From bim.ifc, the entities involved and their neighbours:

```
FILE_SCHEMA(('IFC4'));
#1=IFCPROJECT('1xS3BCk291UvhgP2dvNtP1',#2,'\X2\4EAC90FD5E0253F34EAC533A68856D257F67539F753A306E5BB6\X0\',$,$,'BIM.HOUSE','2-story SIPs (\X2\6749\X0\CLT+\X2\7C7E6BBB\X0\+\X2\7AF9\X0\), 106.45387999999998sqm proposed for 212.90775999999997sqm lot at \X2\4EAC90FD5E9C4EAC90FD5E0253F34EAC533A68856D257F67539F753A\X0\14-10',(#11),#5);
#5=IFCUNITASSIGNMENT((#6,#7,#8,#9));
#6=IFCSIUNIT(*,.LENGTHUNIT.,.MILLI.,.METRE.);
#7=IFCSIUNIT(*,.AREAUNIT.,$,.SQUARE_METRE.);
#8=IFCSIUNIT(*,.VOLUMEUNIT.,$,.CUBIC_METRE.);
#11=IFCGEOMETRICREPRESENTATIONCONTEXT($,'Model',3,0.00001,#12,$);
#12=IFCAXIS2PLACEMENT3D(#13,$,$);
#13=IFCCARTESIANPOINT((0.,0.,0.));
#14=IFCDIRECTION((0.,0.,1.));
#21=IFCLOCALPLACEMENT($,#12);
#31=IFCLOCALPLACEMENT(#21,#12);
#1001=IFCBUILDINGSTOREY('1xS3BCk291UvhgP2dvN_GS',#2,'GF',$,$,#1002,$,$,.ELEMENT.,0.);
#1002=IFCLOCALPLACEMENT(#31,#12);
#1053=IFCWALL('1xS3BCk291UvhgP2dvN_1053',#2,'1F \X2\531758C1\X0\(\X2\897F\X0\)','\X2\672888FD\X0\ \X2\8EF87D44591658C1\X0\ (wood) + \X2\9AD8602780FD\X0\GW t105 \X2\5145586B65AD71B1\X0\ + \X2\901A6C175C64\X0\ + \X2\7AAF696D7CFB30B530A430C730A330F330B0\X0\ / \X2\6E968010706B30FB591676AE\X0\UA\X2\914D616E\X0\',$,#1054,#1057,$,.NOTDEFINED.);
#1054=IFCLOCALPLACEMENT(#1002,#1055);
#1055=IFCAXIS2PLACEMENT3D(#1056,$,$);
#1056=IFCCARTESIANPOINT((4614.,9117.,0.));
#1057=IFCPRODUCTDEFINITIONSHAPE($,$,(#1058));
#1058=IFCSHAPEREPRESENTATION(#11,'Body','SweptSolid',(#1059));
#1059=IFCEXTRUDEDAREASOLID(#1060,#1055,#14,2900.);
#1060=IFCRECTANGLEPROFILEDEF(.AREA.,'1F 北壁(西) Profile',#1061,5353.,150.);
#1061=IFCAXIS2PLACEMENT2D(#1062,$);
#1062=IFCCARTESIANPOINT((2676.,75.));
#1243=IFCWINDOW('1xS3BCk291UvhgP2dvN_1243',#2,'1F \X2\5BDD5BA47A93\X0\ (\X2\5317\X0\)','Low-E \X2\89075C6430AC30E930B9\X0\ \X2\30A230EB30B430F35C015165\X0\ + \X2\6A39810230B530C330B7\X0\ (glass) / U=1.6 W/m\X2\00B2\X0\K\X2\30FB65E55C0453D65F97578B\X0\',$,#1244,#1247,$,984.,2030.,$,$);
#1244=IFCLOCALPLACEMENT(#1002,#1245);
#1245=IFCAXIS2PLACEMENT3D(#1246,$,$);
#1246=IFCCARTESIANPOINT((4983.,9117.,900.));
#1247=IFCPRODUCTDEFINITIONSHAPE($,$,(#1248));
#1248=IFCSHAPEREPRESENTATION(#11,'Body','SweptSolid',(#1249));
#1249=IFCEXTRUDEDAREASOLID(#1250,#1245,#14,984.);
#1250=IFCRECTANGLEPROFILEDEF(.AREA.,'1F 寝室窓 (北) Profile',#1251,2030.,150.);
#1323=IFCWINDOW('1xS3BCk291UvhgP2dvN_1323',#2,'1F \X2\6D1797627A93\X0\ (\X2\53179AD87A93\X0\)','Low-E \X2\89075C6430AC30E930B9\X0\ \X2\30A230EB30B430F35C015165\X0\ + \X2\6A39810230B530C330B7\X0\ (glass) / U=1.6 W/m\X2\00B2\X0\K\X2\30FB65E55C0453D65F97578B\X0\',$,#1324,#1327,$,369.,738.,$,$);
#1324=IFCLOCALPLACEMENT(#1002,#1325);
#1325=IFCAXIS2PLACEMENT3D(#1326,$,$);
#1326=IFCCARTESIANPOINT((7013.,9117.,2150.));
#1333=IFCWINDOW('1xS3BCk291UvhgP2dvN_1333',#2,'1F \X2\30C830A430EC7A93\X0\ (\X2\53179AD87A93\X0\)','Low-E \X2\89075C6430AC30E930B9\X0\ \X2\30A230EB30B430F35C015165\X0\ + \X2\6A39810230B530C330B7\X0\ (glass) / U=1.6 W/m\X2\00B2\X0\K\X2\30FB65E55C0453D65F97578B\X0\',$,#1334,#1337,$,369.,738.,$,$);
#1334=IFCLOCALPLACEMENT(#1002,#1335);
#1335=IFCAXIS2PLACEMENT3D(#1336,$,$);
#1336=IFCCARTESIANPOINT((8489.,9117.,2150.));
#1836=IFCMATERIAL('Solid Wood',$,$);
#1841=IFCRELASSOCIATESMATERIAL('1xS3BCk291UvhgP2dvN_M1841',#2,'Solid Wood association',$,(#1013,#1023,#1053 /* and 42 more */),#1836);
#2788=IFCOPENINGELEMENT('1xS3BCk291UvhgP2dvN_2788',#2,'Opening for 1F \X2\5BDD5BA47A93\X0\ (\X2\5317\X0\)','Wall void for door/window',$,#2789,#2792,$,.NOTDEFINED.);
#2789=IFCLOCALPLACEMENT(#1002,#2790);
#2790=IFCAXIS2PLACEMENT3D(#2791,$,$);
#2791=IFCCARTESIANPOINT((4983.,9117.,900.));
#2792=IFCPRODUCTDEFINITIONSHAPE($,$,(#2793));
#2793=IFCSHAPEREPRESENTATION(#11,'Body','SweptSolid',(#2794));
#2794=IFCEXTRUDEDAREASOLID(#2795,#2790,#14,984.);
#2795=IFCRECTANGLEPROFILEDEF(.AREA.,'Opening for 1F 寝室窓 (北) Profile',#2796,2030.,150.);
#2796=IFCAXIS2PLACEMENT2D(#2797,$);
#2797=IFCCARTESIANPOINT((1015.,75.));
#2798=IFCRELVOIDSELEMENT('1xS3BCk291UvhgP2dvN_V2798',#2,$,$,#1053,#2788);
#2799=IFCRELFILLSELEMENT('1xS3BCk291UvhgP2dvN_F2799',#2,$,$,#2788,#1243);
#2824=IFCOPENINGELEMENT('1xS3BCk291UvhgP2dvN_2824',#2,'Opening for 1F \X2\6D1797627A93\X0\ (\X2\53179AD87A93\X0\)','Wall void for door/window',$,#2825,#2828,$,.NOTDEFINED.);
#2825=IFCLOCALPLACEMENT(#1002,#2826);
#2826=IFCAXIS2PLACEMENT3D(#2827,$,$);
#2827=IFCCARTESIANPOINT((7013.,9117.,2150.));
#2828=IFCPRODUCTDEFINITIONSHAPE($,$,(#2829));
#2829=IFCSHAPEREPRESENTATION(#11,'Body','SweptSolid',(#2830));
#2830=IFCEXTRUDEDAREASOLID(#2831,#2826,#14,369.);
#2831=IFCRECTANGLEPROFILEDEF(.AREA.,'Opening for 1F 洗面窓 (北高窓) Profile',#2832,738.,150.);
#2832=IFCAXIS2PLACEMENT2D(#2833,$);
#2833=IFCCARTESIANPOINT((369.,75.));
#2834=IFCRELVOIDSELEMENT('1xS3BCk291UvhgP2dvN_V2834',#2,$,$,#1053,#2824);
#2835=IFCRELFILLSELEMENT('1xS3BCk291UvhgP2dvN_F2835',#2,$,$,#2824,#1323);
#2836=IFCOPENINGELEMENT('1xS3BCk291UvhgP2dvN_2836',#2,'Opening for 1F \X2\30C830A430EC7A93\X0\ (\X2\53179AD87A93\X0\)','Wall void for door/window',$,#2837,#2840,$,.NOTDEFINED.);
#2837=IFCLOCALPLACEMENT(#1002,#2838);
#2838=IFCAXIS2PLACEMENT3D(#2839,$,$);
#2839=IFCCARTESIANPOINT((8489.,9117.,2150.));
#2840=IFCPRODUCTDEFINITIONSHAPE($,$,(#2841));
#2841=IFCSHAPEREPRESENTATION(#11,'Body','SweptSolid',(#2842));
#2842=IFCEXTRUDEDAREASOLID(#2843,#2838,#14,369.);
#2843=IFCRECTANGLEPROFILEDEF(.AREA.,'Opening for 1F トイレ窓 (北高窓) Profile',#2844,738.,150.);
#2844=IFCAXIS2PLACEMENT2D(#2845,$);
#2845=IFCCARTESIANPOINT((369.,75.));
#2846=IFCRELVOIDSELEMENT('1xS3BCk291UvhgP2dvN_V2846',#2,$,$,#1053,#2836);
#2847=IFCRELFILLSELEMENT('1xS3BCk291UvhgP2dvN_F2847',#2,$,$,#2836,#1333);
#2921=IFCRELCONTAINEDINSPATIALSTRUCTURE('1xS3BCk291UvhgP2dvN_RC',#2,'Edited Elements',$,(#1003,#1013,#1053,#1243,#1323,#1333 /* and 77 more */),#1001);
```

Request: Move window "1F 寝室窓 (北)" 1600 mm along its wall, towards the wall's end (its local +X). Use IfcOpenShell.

```python
import ifcopenshell
import ifcopenshell.api.geometry
import ifcopenshell.util.placement
import ifcopenshell.util.unit

model = ifcopenshell.open("bim.ifc")
unit_scale = ifcopenshell.util.unit.calculate_unit_scale(model)

window = model.by_guid("1xS3BCk291UvhgP2dvN_1243")
opening = window.FillsVoids[0].RelatingOpeningElement
wall = opening.VoidsElements[0].RelatingBuildingElement

wall_matrix = ifcopenshell.util.placement.get_local_placement(wall.ObjectPlacement)
shift = wall_matrix[:3, 0] * 1.6 / unit_scale
before = ifcopenshell.util.placement.get_local_placement(window.ObjectPlacement)[:3, 3].copy()

# The window is not placed relative to its opening, so move both.
for product in (opening, window):
    matrix = ifcopenshell.util.placement.get_local_placement(product.ObjectPlacement)
    matrix[:3, 3] += shift
    ifcopenshell.api.geometry.edit_object_placement(model, product=product, matrix=matrix, is_si=False)

after = ifcopenshell.util.placement.get_local_placement(window.ObjectPlacement)[:3, 3]
print("window moved by", (after - before).round(3) + 0.0)

model.write("bim_updated.ifc")
```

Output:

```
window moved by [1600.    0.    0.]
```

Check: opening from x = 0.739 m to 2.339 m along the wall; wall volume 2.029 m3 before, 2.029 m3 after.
